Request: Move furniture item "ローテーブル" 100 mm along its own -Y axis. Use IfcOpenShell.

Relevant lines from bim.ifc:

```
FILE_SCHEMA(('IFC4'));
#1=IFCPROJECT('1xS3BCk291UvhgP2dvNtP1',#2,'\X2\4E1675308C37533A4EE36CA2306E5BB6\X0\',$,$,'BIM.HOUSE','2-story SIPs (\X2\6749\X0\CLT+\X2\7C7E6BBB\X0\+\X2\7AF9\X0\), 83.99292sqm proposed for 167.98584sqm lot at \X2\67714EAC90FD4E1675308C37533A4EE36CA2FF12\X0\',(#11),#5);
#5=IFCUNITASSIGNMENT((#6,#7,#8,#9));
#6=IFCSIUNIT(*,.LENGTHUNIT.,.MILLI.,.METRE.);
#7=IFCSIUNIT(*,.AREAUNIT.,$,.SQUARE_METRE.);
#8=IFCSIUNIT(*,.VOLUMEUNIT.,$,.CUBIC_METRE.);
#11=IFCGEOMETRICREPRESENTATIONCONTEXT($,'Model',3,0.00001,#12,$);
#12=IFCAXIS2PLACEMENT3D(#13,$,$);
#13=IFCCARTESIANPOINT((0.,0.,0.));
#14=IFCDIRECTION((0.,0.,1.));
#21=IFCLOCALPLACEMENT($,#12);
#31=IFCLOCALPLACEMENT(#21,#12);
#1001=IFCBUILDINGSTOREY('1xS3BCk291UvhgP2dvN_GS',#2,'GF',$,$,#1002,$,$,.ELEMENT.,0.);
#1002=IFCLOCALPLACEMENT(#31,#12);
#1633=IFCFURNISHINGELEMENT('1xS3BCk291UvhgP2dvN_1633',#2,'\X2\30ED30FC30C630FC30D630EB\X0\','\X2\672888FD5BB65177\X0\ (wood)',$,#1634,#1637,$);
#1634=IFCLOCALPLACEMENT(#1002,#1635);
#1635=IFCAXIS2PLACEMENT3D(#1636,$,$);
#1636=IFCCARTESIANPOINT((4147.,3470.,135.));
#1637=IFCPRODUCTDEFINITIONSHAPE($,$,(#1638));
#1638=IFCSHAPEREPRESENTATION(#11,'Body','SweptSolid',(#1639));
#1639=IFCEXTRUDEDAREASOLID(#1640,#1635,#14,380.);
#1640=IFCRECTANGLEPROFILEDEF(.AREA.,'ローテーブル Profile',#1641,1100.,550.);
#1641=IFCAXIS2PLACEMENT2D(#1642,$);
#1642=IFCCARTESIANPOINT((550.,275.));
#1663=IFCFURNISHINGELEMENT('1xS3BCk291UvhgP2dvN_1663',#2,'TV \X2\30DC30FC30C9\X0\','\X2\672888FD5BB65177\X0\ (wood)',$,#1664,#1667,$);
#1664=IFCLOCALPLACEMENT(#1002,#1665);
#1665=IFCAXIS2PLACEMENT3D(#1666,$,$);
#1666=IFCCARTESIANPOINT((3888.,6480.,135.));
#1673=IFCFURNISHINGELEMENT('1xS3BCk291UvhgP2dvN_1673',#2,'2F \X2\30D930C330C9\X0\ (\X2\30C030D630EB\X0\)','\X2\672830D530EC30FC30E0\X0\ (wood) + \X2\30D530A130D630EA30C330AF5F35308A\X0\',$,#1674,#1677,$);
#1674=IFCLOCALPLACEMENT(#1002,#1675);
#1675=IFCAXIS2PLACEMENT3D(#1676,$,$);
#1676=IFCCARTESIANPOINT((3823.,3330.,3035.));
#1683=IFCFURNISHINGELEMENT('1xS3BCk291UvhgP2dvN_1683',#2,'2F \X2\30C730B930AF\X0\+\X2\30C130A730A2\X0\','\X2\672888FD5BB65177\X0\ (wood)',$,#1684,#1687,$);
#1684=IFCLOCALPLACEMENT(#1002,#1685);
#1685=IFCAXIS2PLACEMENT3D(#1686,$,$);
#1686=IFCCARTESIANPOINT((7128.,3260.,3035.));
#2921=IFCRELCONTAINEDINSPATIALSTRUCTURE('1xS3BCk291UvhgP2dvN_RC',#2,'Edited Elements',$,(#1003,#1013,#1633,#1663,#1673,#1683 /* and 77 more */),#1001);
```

```python
import ifcopenshell
import ifcopenshell.api.geometry
import ifcopenshell.util.placement

model = ifcopenshell.open("bim.ifc")

item = model.by_guid("1xS3BCk291UvhgP2dvN_1633")
matrix = ifcopenshell.util.placement.get_local_placement(item.ObjectPlacement)
matrix[:3, 3] -= matrix[:3, 1] * 100.0
ifcopenshell.api.geometry.edit_object_placement(model, product=item, matrix=matrix, is_si=False)

print(ifcopenshell.util.placement.get_local_placement(item.ObjectPlacement).round(3) + 0.0)

model.write("bim_updated.ifc")
```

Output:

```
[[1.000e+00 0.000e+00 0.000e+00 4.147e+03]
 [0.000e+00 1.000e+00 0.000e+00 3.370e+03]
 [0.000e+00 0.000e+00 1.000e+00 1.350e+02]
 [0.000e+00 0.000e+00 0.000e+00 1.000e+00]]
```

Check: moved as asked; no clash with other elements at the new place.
